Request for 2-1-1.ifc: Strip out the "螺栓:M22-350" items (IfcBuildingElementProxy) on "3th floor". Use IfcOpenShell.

First a look at what the model holds.

```python
import ifcopenshell
import ifcopenshell.util.element

model = ifcopenshell.open("2-1-1.ifc")
print(model.schema)
storey = next(s for s in model.by_type("IfcBuildingStorey") if s.Name == "3th floor")
proxies = [e for e in ifcopenshell.util.element.get_decomposition(storey) if e.is_a("IfcBuildingElementProxy")]
seen = {}
for e in proxies:
    element_type = ifcopenshell.util.element.get_type(e)
    name = element_type.Name if element_type not in (None, e) else None
    seen[name] = seen.get(name, 0) + 1
for name, count in sorted(seen.items(), key=str):
    print(count, "x", name)
```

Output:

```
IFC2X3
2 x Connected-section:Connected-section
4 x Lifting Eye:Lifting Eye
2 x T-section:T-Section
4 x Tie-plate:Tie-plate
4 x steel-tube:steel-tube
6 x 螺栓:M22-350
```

```python
import ifcopenshell
import ifcopenshell.api.root
import ifcopenshell.util.element

model = ifcopenshell.open("2-1-1.ifc")

storey = next(s for s in model.by_type("IfcBuildingStorey") if s.Name == "3th floor")
proxies = [e for e in ifcopenshell.util.element.get_decomposition(storey) if e.is_a("IfcBuildingElementProxy")]
targets = [e for e in proxies if (t := ifcopenshell.util.element.get_type(e)) not in (None, e) and t.Name == "螺栓:M22-350"]

for e in targets:
    ifcopenshell.api.root.remove_product(model, product=e)
print(len(targets), "removed")

model.write("2-1-1_edited.ifc")
```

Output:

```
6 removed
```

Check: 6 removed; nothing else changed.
